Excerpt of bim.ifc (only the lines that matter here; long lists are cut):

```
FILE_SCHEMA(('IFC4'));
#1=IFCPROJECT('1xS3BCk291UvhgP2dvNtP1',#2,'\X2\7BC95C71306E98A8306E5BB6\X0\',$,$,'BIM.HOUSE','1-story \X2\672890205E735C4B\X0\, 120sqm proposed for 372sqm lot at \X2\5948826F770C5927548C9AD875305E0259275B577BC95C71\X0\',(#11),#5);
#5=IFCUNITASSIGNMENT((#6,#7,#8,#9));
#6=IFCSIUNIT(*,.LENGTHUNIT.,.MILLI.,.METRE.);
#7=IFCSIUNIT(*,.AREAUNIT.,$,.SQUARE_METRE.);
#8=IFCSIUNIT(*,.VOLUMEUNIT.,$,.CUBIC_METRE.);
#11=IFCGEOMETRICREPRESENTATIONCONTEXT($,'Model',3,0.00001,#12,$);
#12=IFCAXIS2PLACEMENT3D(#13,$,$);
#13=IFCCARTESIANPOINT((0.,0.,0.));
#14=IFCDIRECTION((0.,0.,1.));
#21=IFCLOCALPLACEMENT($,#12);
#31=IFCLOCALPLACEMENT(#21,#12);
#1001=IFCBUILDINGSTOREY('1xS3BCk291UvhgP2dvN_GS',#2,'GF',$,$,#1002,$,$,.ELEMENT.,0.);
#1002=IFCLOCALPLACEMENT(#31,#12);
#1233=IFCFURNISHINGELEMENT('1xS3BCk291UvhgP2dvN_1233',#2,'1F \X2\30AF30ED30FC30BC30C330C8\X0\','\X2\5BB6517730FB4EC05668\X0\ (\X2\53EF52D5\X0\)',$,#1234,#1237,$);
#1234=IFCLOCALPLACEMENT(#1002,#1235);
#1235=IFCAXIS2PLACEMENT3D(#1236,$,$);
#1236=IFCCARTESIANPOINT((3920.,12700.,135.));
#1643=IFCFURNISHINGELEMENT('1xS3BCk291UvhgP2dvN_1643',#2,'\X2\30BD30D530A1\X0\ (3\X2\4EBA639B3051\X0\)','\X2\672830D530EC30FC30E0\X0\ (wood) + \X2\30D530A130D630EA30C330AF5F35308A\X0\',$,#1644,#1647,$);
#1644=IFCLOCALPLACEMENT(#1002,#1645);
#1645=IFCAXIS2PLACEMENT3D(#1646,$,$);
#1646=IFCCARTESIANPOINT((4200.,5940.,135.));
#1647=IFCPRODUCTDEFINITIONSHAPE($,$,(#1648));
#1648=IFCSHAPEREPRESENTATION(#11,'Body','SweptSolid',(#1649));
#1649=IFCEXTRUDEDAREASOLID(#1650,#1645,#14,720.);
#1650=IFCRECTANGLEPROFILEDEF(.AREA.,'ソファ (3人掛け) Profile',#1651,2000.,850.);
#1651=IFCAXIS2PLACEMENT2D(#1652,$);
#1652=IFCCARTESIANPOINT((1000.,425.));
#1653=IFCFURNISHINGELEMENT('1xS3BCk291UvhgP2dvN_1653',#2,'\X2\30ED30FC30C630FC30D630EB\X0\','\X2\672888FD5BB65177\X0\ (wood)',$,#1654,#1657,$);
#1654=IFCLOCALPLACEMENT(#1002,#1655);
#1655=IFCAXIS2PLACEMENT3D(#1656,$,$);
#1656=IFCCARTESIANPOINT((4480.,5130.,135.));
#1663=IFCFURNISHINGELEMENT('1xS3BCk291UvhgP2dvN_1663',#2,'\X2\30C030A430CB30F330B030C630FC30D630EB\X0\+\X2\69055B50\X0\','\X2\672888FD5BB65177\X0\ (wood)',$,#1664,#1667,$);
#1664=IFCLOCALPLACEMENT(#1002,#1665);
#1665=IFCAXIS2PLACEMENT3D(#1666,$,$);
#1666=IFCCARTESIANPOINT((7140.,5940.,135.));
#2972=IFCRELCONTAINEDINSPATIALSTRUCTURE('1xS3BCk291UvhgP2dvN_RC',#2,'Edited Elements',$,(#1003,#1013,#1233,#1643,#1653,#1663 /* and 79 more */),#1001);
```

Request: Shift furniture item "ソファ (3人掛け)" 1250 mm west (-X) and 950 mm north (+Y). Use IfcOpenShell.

```python
import ifcopenshell
import ifcopenshell.api.geometry
import ifcopenshell.util.placement
import ifcopenshell.util.unit

model = ifcopenshell.open("bim.ifc")
unit_scale = ifcopenshell.util.unit.calculate_unit_scale(model)

item = model.by_id(1643)
matrix = ifcopenshell.util.placement.get_local_placement(item.ObjectPlacement)
matrix[0, 3] -= 1.25 / unit_scale
matrix[1, 3] += 0.95 / unit_scale
ifcopenshell.api.geometry.edit_object_placement(model, product=item, matrix=matrix, is_si=False)

print(ifcopenshell.util.placement.get_local_placement(item.ObjectPlacement).round(3) + 0.0)

model.write("bim_rev.ifc")
```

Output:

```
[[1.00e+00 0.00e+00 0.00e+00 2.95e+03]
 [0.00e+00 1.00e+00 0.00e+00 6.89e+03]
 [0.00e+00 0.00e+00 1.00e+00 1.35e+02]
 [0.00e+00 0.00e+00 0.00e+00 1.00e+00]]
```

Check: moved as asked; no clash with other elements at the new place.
